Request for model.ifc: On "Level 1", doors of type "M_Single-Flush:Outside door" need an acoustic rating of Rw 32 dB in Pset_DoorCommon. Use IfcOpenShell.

First a look at what the model holds.

```python
import ifcopenshell
import ifcopenshell.util.element

model = ifcopenshell.open("model.ifc")
print(model.schema)
storey = next(s for s in model.by_type("IfcBuildingStorey") if s.Name == "Level 1")
doors = [e for e in ifcopenshell.util.element.get_decomposition(storey) if e.is_a("IfcDoor")]
seen = {}
for e in doors:
    element_type = ifcopenshell.util.element.get_type(e)
    key = (element_type.Name if element_type != e and element_type else None, ifcopenshell.util.element.get_pset(e, "Pset_DoorCommon", "AcousticRating"))
    seen[key] = seen.get(key, 0) + 1
for (name, value), count in sorted(seen.items(), key=str):
    print(count, "x", name, "|", value)
```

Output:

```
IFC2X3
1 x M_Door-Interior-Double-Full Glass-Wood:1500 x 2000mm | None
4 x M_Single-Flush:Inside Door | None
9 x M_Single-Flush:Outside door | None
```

```python
import ifcopenshell
import ifcopenshell.api.pset
import ifcopenshell.util.element

model = ifcopenshell.open("model.ifc")

storey = next(s for s in model.by_type("IfcBuildingStorey") if s.Name == "Level 1")
doors = [e for e in ifcopenshell.util.element.get_decomposition(storey) if e.is_a("IfcDoor")]

count = 0
for e in doors:
    element_type = ifcopenshell.util.element.get_type(e)
    if element_type in (None, e) or element_type.Name != "M_Single-Flush:Outside door":
        continue
    # add_pset returns the element's existing set when there is one.
    pset = ifcopenshell.api.pset.add_pset(model, product=e, name="Pset_DoorCommon")
    ifcopenshell.api.pset.edit_pset(model, pset=pset, properties={"AcousticRating": "Rw 32 dB"})
    count += 1

print(count, "doors updated")

model.write("model_rev.ifc")
```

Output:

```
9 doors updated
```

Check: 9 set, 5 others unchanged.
